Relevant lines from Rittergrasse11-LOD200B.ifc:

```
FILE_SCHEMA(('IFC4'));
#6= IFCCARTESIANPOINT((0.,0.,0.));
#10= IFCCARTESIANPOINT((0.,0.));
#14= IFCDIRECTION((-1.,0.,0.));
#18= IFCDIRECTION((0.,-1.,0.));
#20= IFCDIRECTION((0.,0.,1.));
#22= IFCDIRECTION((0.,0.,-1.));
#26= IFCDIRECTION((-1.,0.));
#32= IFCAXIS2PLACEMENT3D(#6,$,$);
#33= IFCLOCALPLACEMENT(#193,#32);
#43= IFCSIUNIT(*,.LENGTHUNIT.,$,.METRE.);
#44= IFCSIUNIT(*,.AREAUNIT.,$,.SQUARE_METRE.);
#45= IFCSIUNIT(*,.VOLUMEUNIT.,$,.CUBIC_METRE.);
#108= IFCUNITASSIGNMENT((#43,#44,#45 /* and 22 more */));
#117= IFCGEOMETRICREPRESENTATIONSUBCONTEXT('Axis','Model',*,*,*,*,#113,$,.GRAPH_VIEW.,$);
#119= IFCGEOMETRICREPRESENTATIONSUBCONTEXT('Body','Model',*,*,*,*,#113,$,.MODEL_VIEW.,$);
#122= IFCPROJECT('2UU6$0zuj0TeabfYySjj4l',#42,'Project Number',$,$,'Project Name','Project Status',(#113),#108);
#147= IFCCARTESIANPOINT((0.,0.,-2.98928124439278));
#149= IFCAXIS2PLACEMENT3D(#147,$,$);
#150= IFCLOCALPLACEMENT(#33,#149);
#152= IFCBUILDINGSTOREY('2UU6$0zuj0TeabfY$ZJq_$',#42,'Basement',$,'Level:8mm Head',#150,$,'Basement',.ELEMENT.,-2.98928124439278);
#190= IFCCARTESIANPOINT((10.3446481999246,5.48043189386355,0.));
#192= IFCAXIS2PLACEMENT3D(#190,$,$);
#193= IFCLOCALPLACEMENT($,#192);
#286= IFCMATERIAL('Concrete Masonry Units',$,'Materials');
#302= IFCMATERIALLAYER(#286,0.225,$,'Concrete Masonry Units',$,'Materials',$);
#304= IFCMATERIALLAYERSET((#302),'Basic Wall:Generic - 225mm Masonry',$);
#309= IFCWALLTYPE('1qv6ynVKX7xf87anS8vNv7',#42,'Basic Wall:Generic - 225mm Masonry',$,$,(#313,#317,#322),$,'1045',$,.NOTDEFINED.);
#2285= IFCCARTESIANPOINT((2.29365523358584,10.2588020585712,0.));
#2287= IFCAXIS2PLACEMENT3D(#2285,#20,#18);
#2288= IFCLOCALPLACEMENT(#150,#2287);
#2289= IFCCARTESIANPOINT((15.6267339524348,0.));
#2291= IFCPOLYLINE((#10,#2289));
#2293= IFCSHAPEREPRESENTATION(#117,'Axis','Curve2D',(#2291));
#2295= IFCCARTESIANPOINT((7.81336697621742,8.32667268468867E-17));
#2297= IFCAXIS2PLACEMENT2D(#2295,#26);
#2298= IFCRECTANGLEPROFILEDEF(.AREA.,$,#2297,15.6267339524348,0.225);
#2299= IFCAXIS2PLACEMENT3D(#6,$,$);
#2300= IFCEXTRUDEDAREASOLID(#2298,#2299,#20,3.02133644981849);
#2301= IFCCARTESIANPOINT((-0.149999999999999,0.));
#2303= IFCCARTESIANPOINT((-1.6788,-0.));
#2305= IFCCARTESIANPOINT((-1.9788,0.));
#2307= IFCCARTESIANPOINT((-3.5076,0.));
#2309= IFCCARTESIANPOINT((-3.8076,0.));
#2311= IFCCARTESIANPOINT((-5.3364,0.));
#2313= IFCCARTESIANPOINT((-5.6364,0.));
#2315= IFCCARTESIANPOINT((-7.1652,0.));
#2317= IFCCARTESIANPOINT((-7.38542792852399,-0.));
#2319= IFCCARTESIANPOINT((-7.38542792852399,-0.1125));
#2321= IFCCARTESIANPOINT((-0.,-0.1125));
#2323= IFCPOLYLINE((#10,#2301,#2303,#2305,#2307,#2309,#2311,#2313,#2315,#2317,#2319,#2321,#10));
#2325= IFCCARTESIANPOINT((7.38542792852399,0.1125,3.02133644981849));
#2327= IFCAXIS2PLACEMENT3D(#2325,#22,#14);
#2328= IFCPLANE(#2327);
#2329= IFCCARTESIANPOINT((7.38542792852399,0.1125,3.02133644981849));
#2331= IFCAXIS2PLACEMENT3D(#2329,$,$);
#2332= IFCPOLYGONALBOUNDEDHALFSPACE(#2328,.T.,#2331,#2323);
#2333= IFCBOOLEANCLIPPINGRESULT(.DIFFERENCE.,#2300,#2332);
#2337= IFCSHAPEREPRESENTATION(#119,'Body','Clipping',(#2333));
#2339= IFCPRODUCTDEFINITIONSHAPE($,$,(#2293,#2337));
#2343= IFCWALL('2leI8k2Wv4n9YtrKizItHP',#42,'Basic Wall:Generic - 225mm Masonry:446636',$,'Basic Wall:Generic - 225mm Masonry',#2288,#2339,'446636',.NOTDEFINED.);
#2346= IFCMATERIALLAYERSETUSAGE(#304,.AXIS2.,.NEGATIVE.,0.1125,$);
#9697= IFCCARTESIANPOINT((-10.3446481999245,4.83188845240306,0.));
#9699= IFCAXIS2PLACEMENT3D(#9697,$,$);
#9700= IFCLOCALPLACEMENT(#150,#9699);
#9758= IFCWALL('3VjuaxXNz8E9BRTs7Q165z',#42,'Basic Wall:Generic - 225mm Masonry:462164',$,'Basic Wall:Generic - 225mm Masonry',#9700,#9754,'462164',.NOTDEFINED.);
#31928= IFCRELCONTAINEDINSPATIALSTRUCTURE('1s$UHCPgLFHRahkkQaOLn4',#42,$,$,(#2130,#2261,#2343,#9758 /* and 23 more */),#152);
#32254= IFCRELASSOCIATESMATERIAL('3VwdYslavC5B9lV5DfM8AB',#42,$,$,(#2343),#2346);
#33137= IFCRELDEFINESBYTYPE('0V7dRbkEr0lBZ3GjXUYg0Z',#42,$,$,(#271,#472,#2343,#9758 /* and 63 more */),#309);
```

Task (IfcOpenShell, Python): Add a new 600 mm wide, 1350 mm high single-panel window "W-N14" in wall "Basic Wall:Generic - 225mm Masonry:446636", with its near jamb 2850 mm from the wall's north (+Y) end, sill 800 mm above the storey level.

```python
import numpy as np
import ifcopenshell
import ifcopenshell.api.feature
import ifcopenshell.api.geometry
import ifcopenshell.api.root
import ifcopenshell.api.spatial
import ifcopenshell.geom
import ifcopenshell.util.element
import ifcopenshell.util.placement
import ifcopenshell.util.representation
import ifcopenshell.util.shape
import ifcopenshell.util.unit

model = ifcopenshell.open("Rittergrasse11-LOD200B.ifc")
unit_scale = ifcopenshell.util.unit.calculate_unit_scale(model)
settings = ifcopenshell.geom.settings()


def volume(element):
    """Net volume in cubic metres, openings subtracted."""
    shape = ifcopenshell.geom.create_shape(settings, element)
    return ifcopenshell.util.shape.get_volume(shape.geometry)


wall = model.by_guid("2leI8k2Wv4n9YtrKizItHP")
storey = ifcopenshell.util.element.get_container(wall, ifc_class="IfcBuildingStorey")
context = ifcopenshell.util.representation.get_context(model, "Model", "Body", "MODEL_VIEW")
before = volume(wall)

width, height, from_end, sill = 0.6, 1.35, 2.85, 0.8  # metres

# The wall runs along its own X axis, and the end named is its -X end.
wall_shape = ifcopenshell.geom.create_shape(settings, wall)
x, y, z = ifcopenshell.util.shape.get_vertices(wall_shape.geometry).T
start = x.min() + from_end
face, thickness = float(y.min()), float(y.max() - y.min())
wall_matrix = ifcopenshell.util.placement.get_local_placement(wall.ObjectPlacement)
level = ifcopenshell.util.placement.get_local_placement(storey.ObjectPlacement)[2, 3]


def in_wall(x, y):
    """Placement at x, y metres in the wall's axes, at sill height."""
    matrix = wall_matrix.copy()
    matrix[:, 3] = wall_matrix @ np.array([x / unit_scale, y / unit_scale, 0.0, 1.0])
    matrix[2, 3] = level + sill / unit_scale
    return matrix


# Opening: a box that overshoots both wall faces by 50 mm.
opening = ifcopenshell.api.root.create_entity(model, ifc_class="IfcOpeningElement", predefined_type="OPENING")
box = ifcopenshell.api.geometry.add_wall_representation(
    model, context=context, length=width, height=height, thickness=thickness + 0.1
)
ifcopenshell.api.geometry.assign_representation(model, product=opening, representation=box)
ifcopenshell.api.geometry.edit_object_placement(model, product=opening, matrix=in_wall(start, face - 0.05), is_si=False)
ifcopenshell.api.feature.add_feature(model, feature=opening, element=wall)

window = ifcopenshell.api.root.create_entity(model, ifc_class="IfcWindow", name="W-N14", predefined_type="WINDOW")
window.OverallWidth, window.OverallHeight = width / unit_scale, height / unit_scale
window.PartitioningType = "SINGLE_PANEL"
body = ifcopenshell.api.geometry.add_window_representation(
    model,
    context=context,
    overall_width=window.OverallWidth,
    overall_height=window.OverallHeight,
    partition_type="SINGLE_PANEL",
)
ifcopenshell.api.geometry.assign_representation(model, product=window, representation=body)
ifcopenshell.api.spatial.assign_container(model, products=[window], relating_structure=storey)
ifcopenshell.api.feature.add_filling(model, opening=opening, element=window)

# Centre the window in the wall's thickness.
ifcopenshell.api.geometry.edit_object_placement(model, product=window, matrix=in_wall(start, face), is_si=False)
window_shape = ifcopenshell.geom.create_shape(settings, window)
depth = ifcopenshell.util.shape.get_vertices(window_shape.geometry)[:, 1]
offset = face + thickness / 2 - (depth.min() + depth.max()) / 2
ifcopenshell.api.geometry.edit_object_placement(model, product=window, matrix=in_wall(start, offset), is_si=False)

after = volume(wall)

print(f"wall volume {before:.3f} -> {after:.3f} m3")

model.write("Rittergrasse11-LOD200B_rev.ifc")
```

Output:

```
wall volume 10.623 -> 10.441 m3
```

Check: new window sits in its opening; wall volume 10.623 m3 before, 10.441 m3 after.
